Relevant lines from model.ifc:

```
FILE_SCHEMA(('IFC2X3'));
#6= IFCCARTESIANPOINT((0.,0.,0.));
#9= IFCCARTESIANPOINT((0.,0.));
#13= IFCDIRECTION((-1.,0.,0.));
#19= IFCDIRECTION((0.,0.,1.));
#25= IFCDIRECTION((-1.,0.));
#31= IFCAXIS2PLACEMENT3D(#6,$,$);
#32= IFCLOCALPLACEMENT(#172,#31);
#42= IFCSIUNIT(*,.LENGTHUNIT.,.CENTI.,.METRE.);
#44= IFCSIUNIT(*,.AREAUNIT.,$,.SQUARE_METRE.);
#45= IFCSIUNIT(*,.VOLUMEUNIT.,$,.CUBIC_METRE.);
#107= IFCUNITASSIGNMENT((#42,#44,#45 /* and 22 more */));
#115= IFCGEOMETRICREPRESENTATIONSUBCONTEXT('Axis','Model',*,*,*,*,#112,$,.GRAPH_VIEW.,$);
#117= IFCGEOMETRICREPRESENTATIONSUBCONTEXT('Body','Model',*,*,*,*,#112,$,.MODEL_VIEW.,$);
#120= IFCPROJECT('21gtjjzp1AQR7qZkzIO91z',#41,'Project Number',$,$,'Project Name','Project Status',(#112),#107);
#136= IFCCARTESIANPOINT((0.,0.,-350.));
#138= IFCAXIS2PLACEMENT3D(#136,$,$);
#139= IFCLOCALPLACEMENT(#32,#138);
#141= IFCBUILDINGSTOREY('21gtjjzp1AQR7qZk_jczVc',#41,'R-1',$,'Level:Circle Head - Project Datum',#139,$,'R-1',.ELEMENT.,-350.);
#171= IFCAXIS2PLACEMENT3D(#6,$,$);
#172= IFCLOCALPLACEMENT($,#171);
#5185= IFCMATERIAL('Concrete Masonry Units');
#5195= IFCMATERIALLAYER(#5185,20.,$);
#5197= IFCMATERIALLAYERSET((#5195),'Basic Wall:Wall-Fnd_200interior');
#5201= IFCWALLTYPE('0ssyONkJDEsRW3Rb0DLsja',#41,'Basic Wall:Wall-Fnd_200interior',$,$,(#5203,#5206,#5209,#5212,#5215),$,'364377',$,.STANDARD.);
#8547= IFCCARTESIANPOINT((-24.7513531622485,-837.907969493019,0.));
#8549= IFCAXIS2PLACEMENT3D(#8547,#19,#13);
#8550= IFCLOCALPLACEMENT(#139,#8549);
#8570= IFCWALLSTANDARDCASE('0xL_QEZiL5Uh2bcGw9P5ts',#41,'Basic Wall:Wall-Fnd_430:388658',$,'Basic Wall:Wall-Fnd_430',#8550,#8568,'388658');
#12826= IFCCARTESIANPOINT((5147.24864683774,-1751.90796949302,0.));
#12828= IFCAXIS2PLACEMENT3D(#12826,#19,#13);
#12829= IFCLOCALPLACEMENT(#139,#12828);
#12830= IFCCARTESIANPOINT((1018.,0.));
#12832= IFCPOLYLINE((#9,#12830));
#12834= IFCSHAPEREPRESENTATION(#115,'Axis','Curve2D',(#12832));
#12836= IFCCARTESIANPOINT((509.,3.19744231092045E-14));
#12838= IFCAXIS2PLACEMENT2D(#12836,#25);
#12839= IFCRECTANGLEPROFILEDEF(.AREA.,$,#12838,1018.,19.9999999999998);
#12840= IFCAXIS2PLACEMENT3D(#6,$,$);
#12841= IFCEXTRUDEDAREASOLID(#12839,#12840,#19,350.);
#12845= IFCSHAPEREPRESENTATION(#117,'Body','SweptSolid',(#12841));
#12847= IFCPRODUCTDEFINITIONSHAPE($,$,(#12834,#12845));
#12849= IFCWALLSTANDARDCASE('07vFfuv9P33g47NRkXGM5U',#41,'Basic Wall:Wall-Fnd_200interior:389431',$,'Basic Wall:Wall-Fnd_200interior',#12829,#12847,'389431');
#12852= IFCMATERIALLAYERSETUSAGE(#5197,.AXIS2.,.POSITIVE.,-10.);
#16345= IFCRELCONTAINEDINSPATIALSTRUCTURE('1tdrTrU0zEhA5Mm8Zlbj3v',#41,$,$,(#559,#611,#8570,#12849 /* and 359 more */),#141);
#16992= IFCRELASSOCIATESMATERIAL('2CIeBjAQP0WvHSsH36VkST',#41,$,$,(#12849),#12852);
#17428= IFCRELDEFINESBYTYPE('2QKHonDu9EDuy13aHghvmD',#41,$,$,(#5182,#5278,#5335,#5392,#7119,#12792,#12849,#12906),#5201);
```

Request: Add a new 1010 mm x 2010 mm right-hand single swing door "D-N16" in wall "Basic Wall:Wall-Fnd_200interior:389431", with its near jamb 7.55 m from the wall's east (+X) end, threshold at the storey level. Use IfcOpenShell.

```python
import numpy as np
import ifcopenshell
import ifcopenshell.api.feature
import ifcopenshell.api.geometry
import ifcopenshell.api.root
import ifcopenshell.api.spatial
import ifcopenshell.api.type
import ifcopenshell.geom
import ifcopenshell.util.element
import ifcopenshell.util.placement
import ifcopenshell.util.representation
import ifcopenshell.util.shape
import ifcopenshell.util.unit

model = ifcopenshell.open("model.ifc")
unit_scale = ifcopenshell.util.unit.calculate_unit_scale(model)
settings = ifcopenshell.geom.settings()


def volume(element):
    """Net volume in cubic metres, openings subtracted."""
    shape = ifcopenshell.geom.create_shape(settings, element)
    return ifcopenshell.util.shape.get_volume(shape.geometry)


wall = model.by_guid("07vFfuv9P33g47NRkXGM5U")
storey = ifcopenshell.util.element.get_container(wall, ifc_class="IfcBuildingStorey")
context = ifcopenshell.util.representation.get_context(model, "Model", "Body", "MODEL_VIEW")
before = volume(wall)

width, height, from_end, sill = 1.01, 2.01, 7.55, 0.0  # metres

# The wall runs along its own X axis, and the end named is its -X end.
wall_shape = ifcopenshell.geom.create_shape(settings, wall)
x, y, z = ifcopenshell.util.shape.get_vertices(wall_shape.geometry).T
start = x.min() + from_end
face, thickness = float(y.min()), float(y.max() - y.min())
wall_matrix = ifcopenshell.util.placement.get_local_placement(wall.ObjectPlacement)
level = ifcopenshell.util.placement.get_local_placement(storey.ObjectPlacement)[2, 3]


def in_wall(x, y):
    """Placement at x, y metres in the wall's axes, at sill height."""
    matrix = wall_matrix.copy()
    matrix[:, 3] = wall_matrix @ np.array([x / unit_scale, y / unit_scale, 0.0, 1.0])
    matrix[2, 3] = level + sill / unit_scale
    return matrix


# Opening: a box that overshoots both wall faces by 50 mm.
opening = ifcopenshell.api.root.create_entity(model, ifc_class="IfcOpeningElement")
box = ifcopenshell.api.geometry.add_wall_representation(
    model, context=context, length=width, height=height, thickness=thickness + 0.1
)
ifcopenshell.api.geometry.assign_representation(model, product=opening, representation=box)
ifcopenshell.api.geometry.edit_object_placement(model, product=opening, matrix=in_wall(start, face - 0.05), is_si=False)
ifcopenshell.api.feature.add_feature(model, feature=opening, element=wall)

door = ifcopenshell.api.root.create_entity(model, ifc_class="IfcDoor", name="D-N16")
door.OverallWidth, door.OverallHeight = width / unit_scale, height / unit_scale
body = ifcopenshell.api.geometry.add_door_representation(
    model,
    context=context,
    overall_width=door.OverallWidth,
    overall_height=door.OverallHeight,
    operation_type="SINGLE_SWING_RIGHT",
    lining_properties={"LiningDepth": thickness / unit_scale, "ThresholdDepth": thickness / unit_scale},
)
ifcopenshell.api.geometry.assign_representation(model, product=door, representation=body)
ifcopenshell.api.spatial.assign_container(model, products=[door], relating_structure=storey)
fills = ifcopenshell.api.feature.add_filling(model, opening=opening, element=door)
fills.OwnerHistory = door.OwnerHistory  # required in IFC2X3

# IFC2X3 keeps the operation on the door style.
style = ifcopenshell.api.root.create_entity(model, ifc_class="IfcDoorStyle", name="D-N16")
style.OperationType, style.ConstructionType = "SINGLE_SWING_RIGHT", "NOTDEFINED"
style.ParameterTakesPrecedence = style.Sizeable = False
ifcopenshell.api.type.assign_type(model, related_objects=[door], relating_type=style)

# The lining spans the wall, so the door starts at the wall face.
ifcopenshell.api.geometry.edit_object_placement(model, product=door, matrix=in_wall(start, face), is_si=False)

after = volume(wall)

print(f"wall volume {before:.3f} -> {after:.3f} m3")

model.write("model_v2.ifc")
```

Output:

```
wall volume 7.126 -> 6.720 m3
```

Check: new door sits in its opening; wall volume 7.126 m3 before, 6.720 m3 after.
